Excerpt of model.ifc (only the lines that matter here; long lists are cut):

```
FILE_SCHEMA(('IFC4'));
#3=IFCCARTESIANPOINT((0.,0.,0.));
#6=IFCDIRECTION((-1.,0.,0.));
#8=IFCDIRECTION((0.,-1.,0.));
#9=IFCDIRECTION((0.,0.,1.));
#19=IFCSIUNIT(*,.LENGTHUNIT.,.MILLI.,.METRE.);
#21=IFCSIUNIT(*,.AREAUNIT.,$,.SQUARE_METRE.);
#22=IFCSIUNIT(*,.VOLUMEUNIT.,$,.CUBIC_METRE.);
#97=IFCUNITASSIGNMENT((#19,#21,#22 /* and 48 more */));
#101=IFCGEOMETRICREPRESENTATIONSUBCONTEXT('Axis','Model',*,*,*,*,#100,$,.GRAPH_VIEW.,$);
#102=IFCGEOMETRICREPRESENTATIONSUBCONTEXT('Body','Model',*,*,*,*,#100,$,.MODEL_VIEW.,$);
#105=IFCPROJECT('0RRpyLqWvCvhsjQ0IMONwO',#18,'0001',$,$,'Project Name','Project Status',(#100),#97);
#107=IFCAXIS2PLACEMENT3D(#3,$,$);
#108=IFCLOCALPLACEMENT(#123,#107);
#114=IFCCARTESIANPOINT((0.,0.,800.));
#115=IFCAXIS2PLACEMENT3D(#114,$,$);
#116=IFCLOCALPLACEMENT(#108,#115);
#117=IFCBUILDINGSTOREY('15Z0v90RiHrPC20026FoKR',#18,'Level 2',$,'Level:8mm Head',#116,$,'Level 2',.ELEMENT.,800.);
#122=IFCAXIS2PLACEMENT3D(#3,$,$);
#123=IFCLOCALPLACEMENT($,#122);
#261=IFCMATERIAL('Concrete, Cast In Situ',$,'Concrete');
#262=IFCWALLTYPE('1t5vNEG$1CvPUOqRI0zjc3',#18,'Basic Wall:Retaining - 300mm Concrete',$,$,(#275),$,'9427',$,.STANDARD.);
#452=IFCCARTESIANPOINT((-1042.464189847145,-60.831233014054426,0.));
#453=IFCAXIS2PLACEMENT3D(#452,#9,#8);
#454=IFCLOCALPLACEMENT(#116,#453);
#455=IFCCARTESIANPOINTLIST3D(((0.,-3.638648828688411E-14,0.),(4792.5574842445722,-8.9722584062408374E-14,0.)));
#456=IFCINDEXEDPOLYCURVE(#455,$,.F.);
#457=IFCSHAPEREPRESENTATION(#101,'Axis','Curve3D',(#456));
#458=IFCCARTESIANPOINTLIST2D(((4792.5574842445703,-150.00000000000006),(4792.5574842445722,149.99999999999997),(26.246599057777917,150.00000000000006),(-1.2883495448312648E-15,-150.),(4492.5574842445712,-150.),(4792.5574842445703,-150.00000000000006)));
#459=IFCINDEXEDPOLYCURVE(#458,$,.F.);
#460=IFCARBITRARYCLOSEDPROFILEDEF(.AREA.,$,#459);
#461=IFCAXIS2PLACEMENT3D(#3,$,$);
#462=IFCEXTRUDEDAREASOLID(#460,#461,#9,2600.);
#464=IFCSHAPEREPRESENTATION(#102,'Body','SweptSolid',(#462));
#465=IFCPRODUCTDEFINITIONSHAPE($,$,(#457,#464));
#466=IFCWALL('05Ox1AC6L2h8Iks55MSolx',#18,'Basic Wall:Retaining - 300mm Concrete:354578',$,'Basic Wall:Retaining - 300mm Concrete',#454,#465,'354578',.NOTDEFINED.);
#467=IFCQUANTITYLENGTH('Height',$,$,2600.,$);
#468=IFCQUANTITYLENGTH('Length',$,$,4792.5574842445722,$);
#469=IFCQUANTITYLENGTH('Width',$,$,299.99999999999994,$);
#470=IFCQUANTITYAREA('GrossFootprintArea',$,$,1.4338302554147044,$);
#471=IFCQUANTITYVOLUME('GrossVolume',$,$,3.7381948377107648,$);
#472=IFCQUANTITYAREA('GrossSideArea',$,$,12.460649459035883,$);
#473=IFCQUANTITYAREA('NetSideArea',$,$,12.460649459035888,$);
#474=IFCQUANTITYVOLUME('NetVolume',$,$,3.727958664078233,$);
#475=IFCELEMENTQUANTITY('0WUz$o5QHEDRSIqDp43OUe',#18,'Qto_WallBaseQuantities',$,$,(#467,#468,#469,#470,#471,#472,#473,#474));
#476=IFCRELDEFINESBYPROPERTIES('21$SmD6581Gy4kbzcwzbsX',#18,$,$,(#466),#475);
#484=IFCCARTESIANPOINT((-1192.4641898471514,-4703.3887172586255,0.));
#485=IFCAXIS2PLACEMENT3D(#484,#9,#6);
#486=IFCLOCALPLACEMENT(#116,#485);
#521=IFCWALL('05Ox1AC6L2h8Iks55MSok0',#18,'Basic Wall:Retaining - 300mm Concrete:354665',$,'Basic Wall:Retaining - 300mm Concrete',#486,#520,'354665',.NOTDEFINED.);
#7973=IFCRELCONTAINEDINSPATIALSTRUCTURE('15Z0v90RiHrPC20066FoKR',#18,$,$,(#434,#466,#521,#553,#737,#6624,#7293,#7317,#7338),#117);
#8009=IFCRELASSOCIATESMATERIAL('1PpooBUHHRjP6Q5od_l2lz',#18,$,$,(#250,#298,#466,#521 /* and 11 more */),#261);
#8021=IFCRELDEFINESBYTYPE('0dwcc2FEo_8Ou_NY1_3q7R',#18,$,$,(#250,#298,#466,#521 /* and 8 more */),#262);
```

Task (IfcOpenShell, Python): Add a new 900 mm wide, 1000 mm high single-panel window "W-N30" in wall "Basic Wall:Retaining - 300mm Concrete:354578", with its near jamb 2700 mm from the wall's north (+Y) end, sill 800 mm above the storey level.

```python
import numpy as np
import ifcopenshell
import ifcopenshell.api.feature
import ifcopenshell.api.geometry
import ifcopenshell.api.pset
import ifcopenshell.api.root
import ifcopenshell.api.spatial
import ifcopenshell.geom
import ifcopenshell.util.element
import ifcopenshell.util.placement
import ifcopenshell.util.representation
import ifcopenshell.util.shape
import ifcopenshell.util.unit

model = ifcopenshell.open("model.ifc")
unit_scale = ifcopenshell.util.unit.calculate_unit_scale(model)
area_scale = ifcopenshell.util.unit.calculate_unit_scale(model, "AREAUNIT")
volume_scale = ifcopenshell.util.unit.calculate_unit_scale(model, "VOLUMEUNIT")
settings = ifcopenshell.geom.settings()


def volume(element):
    """Net volume in cubic metres, openings subtracted."""
    shape = ifcopenshell.geom.create_shape(settings, element)
    return ifcopenshell.util.shape.get_volume(shape.geometry)


wall = model.by_id(466)
storey = ifcopenshell.util.element.get_container(wall, ifc_class="IfcBuildingStorey")
context = ifcopenshell.util.representation.get_context(model, "Model", "Body", "MODEL_VIEW")
before = volume(wall)

width, height, from_end, sill = 0.9, 1, 2.7, 0.8  # metres

# The wall runs along its own X axis, and the end named is its -X end.
wall_shape = ifcopenshell.geom.create_shape(settings, wall)
x, y, z = ifcopenshell.util.shape.get_vertices(wall_shape.geometry).T
start = x.min() + from_end
face, thickness = float(y.min()), float(y.max() - y.min())
wall_matrix = ifcopenshell.util.placement.get_local_placement(wall.ObjectPlacement)
level = ifcopenshell.util.placement.get_local_placement(storey.ObjectPlacement)[2, 3]


def in_wall(x, y):
    """Placement at x, y metres in the wall's axes, at sill height."""
    matrix = wall_matrix.copy()
    matrix[:, 3] = wall_matrix @ np.array([x / unit_scale, y / unit_scale, 0.0, 1.0])
    matrix[2, 3] = level + sill / unit_scale
    return matrix


# Opening: a box that overshoots both wall faces by 50 mm.
opening = ifcopenshell.api.root.create_entity(model, ifc_class="IfcOpeningElement", predefined_type="OPENING")
box = ifcopenshell.api.geometry.add_wall_representation(
    model, context=context, length=width, height=height, thickness=thickness + 0.1
)
ifcopenshell.api.geometry.assign_representation(model, product=opening, representation=box)
ifcopenshell.api.geometry.edit_object_placement(model, product=opening, matrix=in_wall(start, face - 0.05), is_si=False)
ifcopenshell.api.feature.add_feature(model, feature=opening, element=wall)

window = ifcopenshell.api.root.create_entity(model, ifc_class="IfcWindow", name="W-N30", predefined_type="WINDOW")
window.OverallWidth, window.OverallHeight = width / unit_scale, height / unit_scale
window.PartitioningType = "SINGLE_PANEL"
body = ifcopenshell.api.geometry.add_window_representation(
    model,
    context=context,
    overall_width=window.OverallWidth,
    overall_height=window.OverallHeight,
    partition_type="SINGLE_PANEL",
)
ifcopenshell.api.geometry.assign_representation(model, product=window, representation=body)
ifcopenshell.api.spatial.assign_container(model, products=[window], relating_structure=storey)
ifcopenshell.api.feature.add_filling(model, opening=opening, element=window)

# Centre the window in the wall's thickness.
ifcopenshell.api.geometry.edit_object_placement(model, product=window, matrix=in_wall(start, face), is_si=False)
window_shape = ifcopenshell.geom.create_shape(settings, window)
depth = ifcopenshell.util.shape.get_vertices(window_shape.geometry)[:, 1]
offset = face + thickness / 2 - (depth.min() + depth.max()) / 2
ifcopenshell.api.geometry.edit_object_placement(model, product=window, matrix=in_wall(start, offset), is_si=False)

after = volume(wall)

# Update the wall's stored quantities.
qto = model.by_id(ifcopenshell.util.element.get_pset(wall, "Qto_WallBaseQuantities", should_inherit=False)["id"])
ifcopenshell.api.pset.edit_qto(model, qto=qto, properties={
    "NetSideArea": after / thickness / area_scale,
    "NetVolume": after / volume_scale,
})

print(f"wall volume {before:.3f} -> {after:.3f} m3")

model.write("model_edited.ifc")
```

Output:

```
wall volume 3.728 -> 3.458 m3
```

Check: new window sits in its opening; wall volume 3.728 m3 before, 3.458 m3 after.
